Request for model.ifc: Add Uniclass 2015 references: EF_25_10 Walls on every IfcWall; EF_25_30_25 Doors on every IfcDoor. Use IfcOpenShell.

First a look at what the model holds.

```python
import ifcopenshell

model = ifcopenshell.open("model.ifc")
print(model.schema)
print("classifications:", [c.Name for c in model.by_type("IfcClassification")])
for ifc_class in ("IfcDoor", "IfcRoof", "IfcStair", "IfcWall", "IfcWindow"):
    print(ifc_class, len(model.by_type(ifc_class)))
```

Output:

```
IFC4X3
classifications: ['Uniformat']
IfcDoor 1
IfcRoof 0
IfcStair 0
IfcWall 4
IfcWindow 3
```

```python
import ifcopenshell
import ifcopenshell.api.classification

model = ifcopenshell.open("model.ifc")

system = ifcopenshell.api.classification.add_classification(model, classification="Uniclass 2015")

codes = {
    "IfcWall": ("EF_25_10", "Walls"),
    "IfcDoor": ("EF_25_30_25", "Doors"),
}
for ifc_class, (code, name) in codes.items():
    products = model.by_type(ifc_class)
    ifcopenshell.api.classification.add_reference(
        model, products=products, classification=system, identification=code, name=name
    )
    print(code, len(products))

model.write("model-out.ifc")
```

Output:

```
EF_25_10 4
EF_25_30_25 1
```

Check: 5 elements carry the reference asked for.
